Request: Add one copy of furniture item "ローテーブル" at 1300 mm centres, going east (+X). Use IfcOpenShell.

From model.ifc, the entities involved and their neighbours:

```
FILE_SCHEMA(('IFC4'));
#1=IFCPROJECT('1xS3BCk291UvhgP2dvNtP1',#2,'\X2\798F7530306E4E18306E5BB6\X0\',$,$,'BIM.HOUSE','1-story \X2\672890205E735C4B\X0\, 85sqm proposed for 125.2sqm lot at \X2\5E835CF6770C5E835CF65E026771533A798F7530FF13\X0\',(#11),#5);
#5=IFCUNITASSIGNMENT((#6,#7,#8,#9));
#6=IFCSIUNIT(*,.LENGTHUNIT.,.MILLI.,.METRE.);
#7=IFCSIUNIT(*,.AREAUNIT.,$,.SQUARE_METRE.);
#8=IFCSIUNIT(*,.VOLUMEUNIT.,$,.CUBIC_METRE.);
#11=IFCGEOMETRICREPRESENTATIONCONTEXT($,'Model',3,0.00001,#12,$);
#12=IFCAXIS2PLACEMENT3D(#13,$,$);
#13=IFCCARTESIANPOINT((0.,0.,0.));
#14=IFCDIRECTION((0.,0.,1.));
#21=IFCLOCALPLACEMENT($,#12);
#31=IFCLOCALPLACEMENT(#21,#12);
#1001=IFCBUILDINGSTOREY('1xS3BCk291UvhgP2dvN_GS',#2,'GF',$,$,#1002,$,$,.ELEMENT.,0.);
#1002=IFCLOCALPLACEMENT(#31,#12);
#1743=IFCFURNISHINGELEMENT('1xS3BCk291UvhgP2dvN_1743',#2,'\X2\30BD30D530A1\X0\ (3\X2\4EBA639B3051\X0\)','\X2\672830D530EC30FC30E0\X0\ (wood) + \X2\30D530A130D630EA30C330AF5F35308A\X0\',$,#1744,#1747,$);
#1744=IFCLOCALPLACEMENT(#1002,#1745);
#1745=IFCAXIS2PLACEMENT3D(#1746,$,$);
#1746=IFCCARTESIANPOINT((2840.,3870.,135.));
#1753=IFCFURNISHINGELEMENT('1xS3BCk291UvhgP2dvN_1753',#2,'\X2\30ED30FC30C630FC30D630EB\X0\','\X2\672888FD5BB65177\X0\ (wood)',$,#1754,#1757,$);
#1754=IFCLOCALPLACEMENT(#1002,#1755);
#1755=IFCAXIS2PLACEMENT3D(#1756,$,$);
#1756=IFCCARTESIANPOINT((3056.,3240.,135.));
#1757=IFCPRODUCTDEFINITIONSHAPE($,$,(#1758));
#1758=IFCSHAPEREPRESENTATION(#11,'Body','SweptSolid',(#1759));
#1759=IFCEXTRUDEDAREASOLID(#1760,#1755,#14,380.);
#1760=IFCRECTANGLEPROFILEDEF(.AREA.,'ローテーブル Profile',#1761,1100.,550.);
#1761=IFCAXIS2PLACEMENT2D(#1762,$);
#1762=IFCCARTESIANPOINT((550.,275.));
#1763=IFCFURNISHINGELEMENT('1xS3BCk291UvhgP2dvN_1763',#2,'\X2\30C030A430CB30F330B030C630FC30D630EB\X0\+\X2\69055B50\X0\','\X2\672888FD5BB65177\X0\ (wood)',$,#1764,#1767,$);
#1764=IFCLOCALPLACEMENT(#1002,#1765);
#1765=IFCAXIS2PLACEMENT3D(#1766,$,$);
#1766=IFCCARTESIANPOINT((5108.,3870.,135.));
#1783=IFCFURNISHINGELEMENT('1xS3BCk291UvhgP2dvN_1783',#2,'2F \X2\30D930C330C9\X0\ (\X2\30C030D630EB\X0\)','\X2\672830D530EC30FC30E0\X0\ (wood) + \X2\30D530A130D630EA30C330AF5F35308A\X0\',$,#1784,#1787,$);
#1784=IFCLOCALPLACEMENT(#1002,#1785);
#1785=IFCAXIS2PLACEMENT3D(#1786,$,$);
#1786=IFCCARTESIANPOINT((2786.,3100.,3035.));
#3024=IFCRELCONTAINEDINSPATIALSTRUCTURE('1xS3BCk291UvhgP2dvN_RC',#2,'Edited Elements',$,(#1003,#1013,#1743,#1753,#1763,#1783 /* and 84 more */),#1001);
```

```python
import numpy as np
import ifcopenshell
import ifcopenshell.api.geometry
import ifcopenshell.api.root
import ifcopenshell.util.element
import ifcopenshell.util.placement

model = ifcopenshell.open("model.ifc")


def reuse_history(source, copy):
    """copy_class also copies each property set's owner history, people and application; keep the originals."""
    for rel in copy.IsDefinedBy:
        if rel.is_a("IfcRelDefinesByProperties") and (history := rel.RelatingPropertyDefinition.OwnerHistory):
            rel.RelatingPropertyDefinition.OwnerHistory = source.OwnerHistory
            ifcopenshell.util.element.remove_deep2(model, history)


source = model.by_guid("1xS3BCk291UvhgP2dvN_1753")
base = ifcopenshell.util.placement.get_local_placement(source.ObjectPlacement)
step = np.array([1.0, 0.0, 0.0]) * 1300.0

for i in range(1, 2):
    copy = ifcopenshell.api.root.copy_class(model, product=source)
    copy.Representation = ifcopenshell.util.element.copy_deep(
        model, source.Representation, exclude=["IfcGeometricRepresentationContext", "IfcRepresentationMap"]
    )
    reuse_history(source, copy)
    matrix = base.copy()
    matrix[:3, 3] += i * step
    print("added at", matrix[:3, 3].round(3) + 0.0)
    ifcopenshell.api.geometry.edit_object_placement(model, product=copy, matrix=matrix, is_si=False)

model.write("model_updated.ifc")
```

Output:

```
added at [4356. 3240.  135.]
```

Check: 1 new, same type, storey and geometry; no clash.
